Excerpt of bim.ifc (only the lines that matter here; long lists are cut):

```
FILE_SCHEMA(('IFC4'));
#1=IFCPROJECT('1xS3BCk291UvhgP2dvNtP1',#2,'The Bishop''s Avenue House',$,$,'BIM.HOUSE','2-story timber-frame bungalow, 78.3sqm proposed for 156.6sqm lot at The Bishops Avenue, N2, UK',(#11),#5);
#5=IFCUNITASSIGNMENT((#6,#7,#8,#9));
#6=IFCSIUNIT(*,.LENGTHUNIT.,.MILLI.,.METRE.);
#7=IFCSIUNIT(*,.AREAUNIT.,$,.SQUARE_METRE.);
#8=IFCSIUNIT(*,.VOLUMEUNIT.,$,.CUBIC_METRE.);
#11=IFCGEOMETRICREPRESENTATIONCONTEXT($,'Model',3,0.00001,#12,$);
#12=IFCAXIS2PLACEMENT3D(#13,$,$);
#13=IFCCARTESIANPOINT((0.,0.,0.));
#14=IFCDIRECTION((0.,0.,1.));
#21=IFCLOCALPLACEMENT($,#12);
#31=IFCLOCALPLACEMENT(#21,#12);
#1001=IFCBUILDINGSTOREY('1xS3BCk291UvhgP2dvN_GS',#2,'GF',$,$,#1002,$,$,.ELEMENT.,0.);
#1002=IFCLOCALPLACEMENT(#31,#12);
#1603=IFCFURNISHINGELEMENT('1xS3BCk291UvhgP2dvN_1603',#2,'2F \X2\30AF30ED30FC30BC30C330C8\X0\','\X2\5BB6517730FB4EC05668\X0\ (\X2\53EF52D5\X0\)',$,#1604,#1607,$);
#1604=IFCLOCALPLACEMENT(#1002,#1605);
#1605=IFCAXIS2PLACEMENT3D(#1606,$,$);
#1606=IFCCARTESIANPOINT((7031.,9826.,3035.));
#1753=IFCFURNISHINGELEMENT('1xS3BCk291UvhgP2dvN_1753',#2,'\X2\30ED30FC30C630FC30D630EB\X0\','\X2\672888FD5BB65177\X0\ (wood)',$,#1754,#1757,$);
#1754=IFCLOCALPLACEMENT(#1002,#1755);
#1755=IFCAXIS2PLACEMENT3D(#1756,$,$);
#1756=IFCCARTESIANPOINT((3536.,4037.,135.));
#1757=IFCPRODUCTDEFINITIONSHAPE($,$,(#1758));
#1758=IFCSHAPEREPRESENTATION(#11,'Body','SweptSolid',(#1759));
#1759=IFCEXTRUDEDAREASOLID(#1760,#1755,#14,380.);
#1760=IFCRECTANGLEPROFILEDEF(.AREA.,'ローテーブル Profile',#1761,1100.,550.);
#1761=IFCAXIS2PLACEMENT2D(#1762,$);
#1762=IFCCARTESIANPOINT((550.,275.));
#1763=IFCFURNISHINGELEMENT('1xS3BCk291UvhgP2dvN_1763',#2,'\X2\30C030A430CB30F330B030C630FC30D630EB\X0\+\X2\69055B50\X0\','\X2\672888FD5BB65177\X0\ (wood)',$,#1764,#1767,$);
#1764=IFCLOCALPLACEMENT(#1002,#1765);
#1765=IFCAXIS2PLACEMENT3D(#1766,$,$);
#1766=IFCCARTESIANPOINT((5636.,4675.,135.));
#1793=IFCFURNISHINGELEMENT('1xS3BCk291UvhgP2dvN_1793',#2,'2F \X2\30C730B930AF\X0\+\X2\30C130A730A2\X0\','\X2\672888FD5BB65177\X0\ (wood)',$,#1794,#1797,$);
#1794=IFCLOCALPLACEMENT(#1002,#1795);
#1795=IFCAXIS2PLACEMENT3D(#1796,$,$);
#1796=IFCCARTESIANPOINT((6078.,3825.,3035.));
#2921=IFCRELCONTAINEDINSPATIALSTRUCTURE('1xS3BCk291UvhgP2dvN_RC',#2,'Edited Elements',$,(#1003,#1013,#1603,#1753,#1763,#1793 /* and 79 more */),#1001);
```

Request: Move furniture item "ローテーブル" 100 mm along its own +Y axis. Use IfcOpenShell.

```python
import ifcopenshell
import ifcopenshell.api.geometry
import ifcopenshell.util.placement
import ifcopenshell.util.unit

model = ifcopenshell.open("bim.ifc")
unit_scale = ifcopenshell.util.unit.calculate_unit_scale(model)

item = model.by_guid("1xS3BCk291UvhgP2dvN_1753")
matrix = ifcopenshell.util.placement.get_local_placement(item.ObjectPlacement)
matrix[:3, 3] += matrix[:3, 1] * 0.1 / unit_scale
ifcopenshell.api.geometry.edit_object_placement(model, product=item, matrix=matrix, is_si=False)

print(ifcopenshell.util.placement.get_local_placement(item.ObjectPlacement).round(3) + 0.0)

model.write("bim_updated.ifc")
```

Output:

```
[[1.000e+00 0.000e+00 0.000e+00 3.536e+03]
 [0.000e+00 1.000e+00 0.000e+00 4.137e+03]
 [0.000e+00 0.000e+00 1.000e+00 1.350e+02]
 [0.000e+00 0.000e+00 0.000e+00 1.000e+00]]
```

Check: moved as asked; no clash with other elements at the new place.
